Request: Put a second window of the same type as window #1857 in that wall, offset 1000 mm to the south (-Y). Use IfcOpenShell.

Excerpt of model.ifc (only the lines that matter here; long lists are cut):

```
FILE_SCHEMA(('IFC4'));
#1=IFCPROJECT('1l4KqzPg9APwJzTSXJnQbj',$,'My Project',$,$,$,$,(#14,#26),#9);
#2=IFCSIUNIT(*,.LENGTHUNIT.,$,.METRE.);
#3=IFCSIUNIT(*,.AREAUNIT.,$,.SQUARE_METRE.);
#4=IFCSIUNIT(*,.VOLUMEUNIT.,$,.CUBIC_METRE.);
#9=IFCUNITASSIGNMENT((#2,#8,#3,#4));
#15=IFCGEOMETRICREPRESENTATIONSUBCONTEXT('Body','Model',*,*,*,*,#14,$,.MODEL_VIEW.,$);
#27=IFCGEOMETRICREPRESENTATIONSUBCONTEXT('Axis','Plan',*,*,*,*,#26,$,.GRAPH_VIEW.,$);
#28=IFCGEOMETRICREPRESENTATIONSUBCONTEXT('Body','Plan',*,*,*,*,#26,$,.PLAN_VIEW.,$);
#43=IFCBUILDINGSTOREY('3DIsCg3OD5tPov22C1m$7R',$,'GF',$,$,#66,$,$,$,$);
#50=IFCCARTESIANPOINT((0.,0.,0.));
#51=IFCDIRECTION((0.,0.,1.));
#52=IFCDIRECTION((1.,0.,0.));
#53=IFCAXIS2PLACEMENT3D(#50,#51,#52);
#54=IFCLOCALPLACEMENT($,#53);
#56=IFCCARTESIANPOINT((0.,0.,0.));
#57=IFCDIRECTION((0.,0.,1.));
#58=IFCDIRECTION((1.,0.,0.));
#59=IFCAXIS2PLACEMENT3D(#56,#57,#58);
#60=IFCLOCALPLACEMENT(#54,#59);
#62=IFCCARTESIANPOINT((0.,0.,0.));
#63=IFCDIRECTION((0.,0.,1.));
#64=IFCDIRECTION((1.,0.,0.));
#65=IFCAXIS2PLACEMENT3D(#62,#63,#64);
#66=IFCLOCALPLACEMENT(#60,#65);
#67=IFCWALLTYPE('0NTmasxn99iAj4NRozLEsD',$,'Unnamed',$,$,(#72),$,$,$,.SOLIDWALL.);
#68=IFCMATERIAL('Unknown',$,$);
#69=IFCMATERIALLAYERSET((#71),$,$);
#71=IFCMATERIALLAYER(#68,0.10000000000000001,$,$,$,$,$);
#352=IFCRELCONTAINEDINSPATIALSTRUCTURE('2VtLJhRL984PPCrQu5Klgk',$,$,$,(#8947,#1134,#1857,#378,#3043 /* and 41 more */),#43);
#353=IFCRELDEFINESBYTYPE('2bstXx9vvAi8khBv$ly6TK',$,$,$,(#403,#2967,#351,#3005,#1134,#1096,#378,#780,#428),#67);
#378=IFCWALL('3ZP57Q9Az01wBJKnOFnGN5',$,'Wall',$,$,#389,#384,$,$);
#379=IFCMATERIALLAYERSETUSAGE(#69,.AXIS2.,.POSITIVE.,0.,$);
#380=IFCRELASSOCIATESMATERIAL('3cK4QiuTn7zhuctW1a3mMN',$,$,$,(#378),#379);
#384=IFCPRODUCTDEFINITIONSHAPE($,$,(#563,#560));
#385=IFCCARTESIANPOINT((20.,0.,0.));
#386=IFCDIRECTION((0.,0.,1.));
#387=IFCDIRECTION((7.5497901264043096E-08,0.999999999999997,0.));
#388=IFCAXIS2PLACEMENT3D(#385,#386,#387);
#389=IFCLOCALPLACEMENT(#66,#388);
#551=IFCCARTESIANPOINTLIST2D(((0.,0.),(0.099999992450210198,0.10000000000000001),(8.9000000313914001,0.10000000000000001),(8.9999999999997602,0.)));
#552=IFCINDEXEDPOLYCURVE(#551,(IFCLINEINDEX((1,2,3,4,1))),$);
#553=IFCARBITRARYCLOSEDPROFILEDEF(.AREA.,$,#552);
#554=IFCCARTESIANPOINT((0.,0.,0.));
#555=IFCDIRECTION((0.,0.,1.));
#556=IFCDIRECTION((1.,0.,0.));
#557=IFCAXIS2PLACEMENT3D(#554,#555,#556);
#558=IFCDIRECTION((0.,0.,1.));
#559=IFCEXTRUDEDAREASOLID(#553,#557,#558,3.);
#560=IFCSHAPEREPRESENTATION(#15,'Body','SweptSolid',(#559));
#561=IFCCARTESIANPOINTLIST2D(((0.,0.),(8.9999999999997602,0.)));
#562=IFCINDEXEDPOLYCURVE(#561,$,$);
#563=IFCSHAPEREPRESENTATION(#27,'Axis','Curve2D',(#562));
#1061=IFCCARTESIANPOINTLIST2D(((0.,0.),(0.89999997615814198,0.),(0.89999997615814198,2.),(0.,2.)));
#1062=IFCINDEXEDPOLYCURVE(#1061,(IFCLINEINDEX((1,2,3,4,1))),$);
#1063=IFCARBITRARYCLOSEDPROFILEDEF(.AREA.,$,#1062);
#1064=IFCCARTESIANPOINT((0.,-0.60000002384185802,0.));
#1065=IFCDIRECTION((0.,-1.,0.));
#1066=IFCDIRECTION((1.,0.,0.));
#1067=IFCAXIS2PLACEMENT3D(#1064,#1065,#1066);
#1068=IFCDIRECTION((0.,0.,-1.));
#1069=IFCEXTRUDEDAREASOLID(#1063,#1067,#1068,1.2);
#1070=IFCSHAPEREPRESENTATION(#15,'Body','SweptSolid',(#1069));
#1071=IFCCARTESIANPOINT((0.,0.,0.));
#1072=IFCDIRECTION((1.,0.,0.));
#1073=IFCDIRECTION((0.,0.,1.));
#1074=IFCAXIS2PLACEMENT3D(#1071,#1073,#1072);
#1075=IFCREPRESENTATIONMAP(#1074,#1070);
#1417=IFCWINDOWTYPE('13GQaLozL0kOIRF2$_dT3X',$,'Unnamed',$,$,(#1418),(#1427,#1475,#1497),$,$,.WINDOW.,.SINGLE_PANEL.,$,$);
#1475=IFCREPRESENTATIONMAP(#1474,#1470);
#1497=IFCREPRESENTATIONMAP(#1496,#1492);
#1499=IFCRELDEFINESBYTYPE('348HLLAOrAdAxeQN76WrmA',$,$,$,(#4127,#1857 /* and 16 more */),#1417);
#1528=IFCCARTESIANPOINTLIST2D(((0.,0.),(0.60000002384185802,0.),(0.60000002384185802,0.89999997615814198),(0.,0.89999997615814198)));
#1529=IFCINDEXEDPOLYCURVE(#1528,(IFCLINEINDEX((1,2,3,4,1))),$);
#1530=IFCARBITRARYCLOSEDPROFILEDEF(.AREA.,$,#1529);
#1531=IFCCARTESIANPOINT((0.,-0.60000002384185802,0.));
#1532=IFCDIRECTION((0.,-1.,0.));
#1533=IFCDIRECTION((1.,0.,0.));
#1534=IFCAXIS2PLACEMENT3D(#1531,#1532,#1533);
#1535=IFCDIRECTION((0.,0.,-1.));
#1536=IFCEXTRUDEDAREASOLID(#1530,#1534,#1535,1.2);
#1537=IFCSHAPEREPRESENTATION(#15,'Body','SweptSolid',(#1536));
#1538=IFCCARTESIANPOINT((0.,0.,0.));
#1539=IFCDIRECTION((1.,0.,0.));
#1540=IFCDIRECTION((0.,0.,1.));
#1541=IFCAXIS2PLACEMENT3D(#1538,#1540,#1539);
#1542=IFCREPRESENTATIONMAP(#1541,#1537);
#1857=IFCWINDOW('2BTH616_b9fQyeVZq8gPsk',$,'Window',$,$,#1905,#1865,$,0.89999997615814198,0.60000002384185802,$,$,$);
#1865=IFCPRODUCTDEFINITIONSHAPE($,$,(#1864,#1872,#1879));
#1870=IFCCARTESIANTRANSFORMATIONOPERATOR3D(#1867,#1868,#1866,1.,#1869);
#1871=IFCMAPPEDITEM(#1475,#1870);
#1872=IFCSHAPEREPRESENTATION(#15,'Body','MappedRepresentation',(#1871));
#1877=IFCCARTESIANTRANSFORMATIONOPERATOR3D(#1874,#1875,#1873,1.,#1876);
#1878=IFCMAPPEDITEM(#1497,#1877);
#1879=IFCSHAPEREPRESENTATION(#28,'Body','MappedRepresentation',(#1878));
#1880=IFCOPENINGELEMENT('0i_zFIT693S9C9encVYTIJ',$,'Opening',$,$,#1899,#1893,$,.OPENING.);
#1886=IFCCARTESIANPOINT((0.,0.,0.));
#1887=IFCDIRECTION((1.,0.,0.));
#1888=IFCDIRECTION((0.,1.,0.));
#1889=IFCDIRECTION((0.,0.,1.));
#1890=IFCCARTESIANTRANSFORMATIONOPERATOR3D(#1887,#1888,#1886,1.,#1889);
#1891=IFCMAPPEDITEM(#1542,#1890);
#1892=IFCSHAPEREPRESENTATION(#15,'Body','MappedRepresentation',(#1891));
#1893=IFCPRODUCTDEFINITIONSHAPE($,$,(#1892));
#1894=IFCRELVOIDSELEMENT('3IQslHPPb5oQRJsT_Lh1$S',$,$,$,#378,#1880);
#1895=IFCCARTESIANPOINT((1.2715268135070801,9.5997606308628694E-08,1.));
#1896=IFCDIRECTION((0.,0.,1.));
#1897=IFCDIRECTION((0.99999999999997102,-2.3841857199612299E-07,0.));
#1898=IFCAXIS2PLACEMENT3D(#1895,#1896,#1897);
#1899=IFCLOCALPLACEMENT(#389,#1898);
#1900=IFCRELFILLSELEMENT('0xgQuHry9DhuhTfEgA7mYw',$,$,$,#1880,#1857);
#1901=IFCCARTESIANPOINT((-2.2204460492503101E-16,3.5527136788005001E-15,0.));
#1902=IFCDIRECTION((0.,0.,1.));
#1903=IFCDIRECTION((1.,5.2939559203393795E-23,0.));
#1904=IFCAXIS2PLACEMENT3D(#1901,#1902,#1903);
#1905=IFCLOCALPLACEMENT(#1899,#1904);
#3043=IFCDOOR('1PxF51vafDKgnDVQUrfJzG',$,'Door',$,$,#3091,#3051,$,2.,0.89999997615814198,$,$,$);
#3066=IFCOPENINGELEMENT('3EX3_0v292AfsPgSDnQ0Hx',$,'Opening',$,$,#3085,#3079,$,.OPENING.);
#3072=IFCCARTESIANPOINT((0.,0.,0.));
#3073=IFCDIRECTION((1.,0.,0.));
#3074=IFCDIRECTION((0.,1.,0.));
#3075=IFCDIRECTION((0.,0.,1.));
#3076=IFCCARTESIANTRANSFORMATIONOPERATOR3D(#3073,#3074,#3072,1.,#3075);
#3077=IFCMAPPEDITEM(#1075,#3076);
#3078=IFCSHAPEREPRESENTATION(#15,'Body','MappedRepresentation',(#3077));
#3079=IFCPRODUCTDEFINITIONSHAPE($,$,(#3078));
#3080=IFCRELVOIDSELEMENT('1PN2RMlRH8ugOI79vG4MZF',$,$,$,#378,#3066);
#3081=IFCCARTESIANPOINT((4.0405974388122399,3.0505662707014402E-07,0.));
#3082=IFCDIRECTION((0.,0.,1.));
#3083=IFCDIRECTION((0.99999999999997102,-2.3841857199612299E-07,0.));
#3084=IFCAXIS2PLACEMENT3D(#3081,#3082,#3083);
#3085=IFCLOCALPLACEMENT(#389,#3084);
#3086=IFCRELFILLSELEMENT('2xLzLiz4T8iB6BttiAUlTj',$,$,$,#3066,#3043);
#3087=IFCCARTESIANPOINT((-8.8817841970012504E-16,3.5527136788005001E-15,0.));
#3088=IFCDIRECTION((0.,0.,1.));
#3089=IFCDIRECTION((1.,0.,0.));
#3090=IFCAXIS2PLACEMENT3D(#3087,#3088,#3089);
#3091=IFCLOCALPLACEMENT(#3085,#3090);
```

```python
import ifcopenshell
import ifcopenshell.api.feature
import ifcopenshell.api.geometry
import ifcopenshell.api.root
import ifcopenshell.geom
import ifcopenshell.util.element
import ifcopenshell.util.placement
import ifcopenshell.util.shape
import ifcopenshell.util.unit

model = ifcopenshell.open("model.ifc")
unit_scale = ifcopenshell.util.unit.calculate_unit_scale(model)
settings = ifcopenshell.geom.settings()


def volume(element):
    """Net volume in cubic metres, openings subtracted."""
    shape = ifcopenshell.geom.create_shape(settings, element)
    return ifcopenshell.util.shape.get_volume(shape.geometry)


window = model.by_id(1857)
opening = window.FillsVoids[0].RelatingOpeningElement
wall = opening.VoidsElements[0].RelatingBuildingElement
before = volume(wall)
shift = ifcopenshell.util.placement.get_local_placement(wall.ObjectPlacement)[:3, 0] * -1 / unit_scale

# copy_class copies the void relationship, type, container and properties, but no geometry.
new_opening = ifcopenshell.api.root.copy_class(model, product=opening)
new_opening.Representation = ifcopenshell.util.element.copy_deep(
    model, opening.Representation, exclude=["IfcGeometricRepresentationContext", "IfcRepresentationMap"]
)
new_window = ifcopenshell.api.root.copy_class(model, product=window)
new_window.Representation = ifcopenshell.util.element.copy_deep(
    model, window.Representation, exclude=["IfcGeometricRepresentationContext", "IfcRepresentationMap"]
)
ifcopenshell.api.feature.add_filling(model, opening=new_opening, element=new_window)

for old, new in ((opening, new_opening), (window, new_window)):
    matrix = ifcopenshell.util.placement.get_local_placement(old.ObjectPlacement)
    matrix[:3, 3] += shift
    ifcopenshell.api.geometry.edit_object_placement(model, product=new, matrix=matrix, is_si=False)

after = volume(wall)

print(f"wall volume {before:.3f} -> {after:.3f} m3")

model.write("model_v2.ifc")
```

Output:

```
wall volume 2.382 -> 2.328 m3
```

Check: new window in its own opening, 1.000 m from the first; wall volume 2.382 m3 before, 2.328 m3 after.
